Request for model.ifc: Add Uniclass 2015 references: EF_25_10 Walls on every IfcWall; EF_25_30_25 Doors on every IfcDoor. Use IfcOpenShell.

First a look at what the model holds.

```python
import ifcopenshell

model = ifcopenshell.open("model.ifc")
print(model.schema)
print("classifications:", [c.Name for c in model.by_type("IfcClassification")])
for ifc_class in ("IfcDoor", "IfcRoof", "IfcStair", "IfcWall", "IfcWindow"):
    print(ifc_class, len(model.by_type(ifc_class)))
```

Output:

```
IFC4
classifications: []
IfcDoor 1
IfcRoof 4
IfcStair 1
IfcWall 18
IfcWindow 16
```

```python
import ifcopenshell
import ifcopenshell.api.classification

model = ifcopenshell.open("model.ifc")

system = ifcopenshell.api.classification.add_classification(model, classification="Uniclass 2015")

codes = {
    "IfcWall": ("EF_25_10", "Walls"),
    "IfcDoor": ("EF_25_30_25", "Doors"),
}
for ifc_class, (code, name) in codes.items():
    products = model.by_type(ifc_class)
    ifcopenshell.api.classification.add_reference(
        model, products=products, classification=system, identification=code, name=name
    )
    print(code, len(products))

model.write("model_v2.ifc")
```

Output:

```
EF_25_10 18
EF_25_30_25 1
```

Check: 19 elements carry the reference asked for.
